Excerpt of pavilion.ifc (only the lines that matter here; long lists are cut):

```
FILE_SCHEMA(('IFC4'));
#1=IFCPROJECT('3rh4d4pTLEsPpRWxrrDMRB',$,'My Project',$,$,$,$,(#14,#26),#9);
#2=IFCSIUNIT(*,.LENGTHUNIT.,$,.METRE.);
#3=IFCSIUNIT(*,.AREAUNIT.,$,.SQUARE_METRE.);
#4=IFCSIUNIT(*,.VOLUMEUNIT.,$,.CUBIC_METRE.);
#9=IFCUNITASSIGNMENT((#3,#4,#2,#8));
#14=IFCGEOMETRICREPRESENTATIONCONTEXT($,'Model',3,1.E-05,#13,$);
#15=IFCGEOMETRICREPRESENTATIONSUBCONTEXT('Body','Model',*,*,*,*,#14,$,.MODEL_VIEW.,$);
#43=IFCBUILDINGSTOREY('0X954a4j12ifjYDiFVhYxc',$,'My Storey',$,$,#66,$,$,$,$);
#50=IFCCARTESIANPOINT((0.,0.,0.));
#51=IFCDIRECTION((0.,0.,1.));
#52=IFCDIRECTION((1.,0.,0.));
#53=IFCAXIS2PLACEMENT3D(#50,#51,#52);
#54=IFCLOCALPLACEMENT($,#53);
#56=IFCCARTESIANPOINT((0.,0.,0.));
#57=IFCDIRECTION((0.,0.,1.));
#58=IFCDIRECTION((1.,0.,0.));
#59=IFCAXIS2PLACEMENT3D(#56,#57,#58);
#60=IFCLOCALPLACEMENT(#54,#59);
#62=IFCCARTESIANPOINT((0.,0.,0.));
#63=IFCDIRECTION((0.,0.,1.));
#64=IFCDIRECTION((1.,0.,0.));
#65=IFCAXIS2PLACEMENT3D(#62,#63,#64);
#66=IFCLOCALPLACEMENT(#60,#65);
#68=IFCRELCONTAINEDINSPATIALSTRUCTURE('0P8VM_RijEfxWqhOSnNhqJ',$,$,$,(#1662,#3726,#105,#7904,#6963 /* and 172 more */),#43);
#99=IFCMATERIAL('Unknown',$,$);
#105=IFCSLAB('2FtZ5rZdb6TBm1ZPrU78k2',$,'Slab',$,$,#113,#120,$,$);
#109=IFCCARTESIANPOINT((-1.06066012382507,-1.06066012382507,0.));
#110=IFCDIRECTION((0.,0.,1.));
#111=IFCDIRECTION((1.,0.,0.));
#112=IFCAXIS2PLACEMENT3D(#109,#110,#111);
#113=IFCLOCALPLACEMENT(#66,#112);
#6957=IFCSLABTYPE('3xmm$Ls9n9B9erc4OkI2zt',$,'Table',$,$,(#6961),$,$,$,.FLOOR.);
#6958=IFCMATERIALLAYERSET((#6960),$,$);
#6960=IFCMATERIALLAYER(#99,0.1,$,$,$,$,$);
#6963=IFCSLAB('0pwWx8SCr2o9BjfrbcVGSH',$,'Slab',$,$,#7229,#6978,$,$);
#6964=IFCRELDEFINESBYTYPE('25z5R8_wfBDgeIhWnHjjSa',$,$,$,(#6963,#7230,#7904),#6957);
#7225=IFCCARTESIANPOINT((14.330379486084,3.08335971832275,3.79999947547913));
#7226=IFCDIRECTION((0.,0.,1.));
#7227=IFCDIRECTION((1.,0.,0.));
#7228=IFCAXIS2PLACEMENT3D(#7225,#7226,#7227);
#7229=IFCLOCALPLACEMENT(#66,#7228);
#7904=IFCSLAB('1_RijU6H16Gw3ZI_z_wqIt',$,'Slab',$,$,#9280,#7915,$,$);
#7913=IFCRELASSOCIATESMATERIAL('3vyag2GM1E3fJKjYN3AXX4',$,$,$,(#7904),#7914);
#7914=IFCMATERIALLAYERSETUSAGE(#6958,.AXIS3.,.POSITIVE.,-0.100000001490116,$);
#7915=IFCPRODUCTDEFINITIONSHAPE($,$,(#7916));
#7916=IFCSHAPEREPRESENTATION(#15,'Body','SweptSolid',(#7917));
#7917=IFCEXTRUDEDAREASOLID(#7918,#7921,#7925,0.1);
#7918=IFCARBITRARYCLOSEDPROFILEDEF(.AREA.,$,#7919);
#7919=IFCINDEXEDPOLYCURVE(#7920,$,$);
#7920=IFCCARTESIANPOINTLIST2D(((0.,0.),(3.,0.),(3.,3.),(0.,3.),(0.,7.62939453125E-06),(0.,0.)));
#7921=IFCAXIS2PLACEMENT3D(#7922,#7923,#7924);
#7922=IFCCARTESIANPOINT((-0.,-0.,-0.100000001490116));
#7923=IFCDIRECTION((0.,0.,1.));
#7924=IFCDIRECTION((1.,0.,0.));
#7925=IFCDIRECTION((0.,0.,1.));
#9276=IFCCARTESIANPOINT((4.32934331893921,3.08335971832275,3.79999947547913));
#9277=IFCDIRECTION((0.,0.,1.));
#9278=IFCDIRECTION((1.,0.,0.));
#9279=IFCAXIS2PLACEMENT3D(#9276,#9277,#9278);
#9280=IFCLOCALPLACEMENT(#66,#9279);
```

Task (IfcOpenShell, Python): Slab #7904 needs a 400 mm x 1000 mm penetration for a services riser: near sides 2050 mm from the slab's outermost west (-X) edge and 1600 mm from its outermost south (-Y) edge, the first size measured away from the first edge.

```python
import numpy as np
import ifcopenshell
import ifcopenshell.api.feature
import ifcopenshell.api.geometry
import ifcopenshell.api.root
import ifcopenshell.geom
import ifcopenshell.util.placement
import ifcopenshell.util.representation
import ifcopenshell.util.shape
import ifcopenshell.util.unit

model = ifcopenshell.open("pavilion.ifc")
unit_scale = ifcopenshell.util.unit.calculate_unit_scale(model)
settings = ifcopenshell.geom.settings()


def volume(element):
    """Net volume in cubic metres, openings subtracted."""
    shape = ifcopenshell.geom.create_shape(settings, element)
    return ifcopenshell.util.shape.get_volume(shape.geometry)


slab = model.by_guid("1_RijU6H16Gw3ZI_z_wqIt")
before = volume(slab)

# Extent in the slab's own axes, in metres. The edges named are its -X and -Y sides.
slab_shape = ifcopenshell.geom.create_shape(settings, slab)
vertices = ifcopenshell.util.shape.get_vertices(slab_shape.geometry)
x_min, y_min, bottom = vertices.min(axis=0)
top = vertices[:, 2].max()

opening = ifcopenshell.api.root.create_entity(model, ifc_class="IfcOpeningElement", name="Services riser opening", predefined_type="OPENING")
context = ifcopenshell.util.representation.get_context(model, "Model", "Body", "MODEL_VIEW")
width, depth = 0.4, 1
outline = [(0.0, 0.0), (width, 0.0), (width, depth), (0.0, depth), (0.0, 0.0)]
# Overshoot both faces by 50 mm so the cut is clean.
shape = ifcopenshell.api.geometry.add_slab_representation(
    model, context=context, depth=top - bottom + 0.1, polyline=outline
)
ifcopenshell.api.geometry.assign_representation(model, product=opening, representation=shape)

matrix = ifcopenshell.util.placement.get_local_placement(slab.ObjectPlacement)
matrix[:, 3] = matrix @ np.append(np.array([x_min + 2.05, y_min + 1.6, bottom - 0.05]) / unit_scale, 1.0)
ifcopenshell.api.geometry.edit_object_placement(model, product=opening, matrix=matrix, is_si=False)
ifcopenshell.api.feature.add_feature(model, feature=opening, element=slab)

after = volume(slab)

print(f"slab volume {before:.3f} -> {after:.3f} m3")

model.write("pavilion_updated.ifc")
```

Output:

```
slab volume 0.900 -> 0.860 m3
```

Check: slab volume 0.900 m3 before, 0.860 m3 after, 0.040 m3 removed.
